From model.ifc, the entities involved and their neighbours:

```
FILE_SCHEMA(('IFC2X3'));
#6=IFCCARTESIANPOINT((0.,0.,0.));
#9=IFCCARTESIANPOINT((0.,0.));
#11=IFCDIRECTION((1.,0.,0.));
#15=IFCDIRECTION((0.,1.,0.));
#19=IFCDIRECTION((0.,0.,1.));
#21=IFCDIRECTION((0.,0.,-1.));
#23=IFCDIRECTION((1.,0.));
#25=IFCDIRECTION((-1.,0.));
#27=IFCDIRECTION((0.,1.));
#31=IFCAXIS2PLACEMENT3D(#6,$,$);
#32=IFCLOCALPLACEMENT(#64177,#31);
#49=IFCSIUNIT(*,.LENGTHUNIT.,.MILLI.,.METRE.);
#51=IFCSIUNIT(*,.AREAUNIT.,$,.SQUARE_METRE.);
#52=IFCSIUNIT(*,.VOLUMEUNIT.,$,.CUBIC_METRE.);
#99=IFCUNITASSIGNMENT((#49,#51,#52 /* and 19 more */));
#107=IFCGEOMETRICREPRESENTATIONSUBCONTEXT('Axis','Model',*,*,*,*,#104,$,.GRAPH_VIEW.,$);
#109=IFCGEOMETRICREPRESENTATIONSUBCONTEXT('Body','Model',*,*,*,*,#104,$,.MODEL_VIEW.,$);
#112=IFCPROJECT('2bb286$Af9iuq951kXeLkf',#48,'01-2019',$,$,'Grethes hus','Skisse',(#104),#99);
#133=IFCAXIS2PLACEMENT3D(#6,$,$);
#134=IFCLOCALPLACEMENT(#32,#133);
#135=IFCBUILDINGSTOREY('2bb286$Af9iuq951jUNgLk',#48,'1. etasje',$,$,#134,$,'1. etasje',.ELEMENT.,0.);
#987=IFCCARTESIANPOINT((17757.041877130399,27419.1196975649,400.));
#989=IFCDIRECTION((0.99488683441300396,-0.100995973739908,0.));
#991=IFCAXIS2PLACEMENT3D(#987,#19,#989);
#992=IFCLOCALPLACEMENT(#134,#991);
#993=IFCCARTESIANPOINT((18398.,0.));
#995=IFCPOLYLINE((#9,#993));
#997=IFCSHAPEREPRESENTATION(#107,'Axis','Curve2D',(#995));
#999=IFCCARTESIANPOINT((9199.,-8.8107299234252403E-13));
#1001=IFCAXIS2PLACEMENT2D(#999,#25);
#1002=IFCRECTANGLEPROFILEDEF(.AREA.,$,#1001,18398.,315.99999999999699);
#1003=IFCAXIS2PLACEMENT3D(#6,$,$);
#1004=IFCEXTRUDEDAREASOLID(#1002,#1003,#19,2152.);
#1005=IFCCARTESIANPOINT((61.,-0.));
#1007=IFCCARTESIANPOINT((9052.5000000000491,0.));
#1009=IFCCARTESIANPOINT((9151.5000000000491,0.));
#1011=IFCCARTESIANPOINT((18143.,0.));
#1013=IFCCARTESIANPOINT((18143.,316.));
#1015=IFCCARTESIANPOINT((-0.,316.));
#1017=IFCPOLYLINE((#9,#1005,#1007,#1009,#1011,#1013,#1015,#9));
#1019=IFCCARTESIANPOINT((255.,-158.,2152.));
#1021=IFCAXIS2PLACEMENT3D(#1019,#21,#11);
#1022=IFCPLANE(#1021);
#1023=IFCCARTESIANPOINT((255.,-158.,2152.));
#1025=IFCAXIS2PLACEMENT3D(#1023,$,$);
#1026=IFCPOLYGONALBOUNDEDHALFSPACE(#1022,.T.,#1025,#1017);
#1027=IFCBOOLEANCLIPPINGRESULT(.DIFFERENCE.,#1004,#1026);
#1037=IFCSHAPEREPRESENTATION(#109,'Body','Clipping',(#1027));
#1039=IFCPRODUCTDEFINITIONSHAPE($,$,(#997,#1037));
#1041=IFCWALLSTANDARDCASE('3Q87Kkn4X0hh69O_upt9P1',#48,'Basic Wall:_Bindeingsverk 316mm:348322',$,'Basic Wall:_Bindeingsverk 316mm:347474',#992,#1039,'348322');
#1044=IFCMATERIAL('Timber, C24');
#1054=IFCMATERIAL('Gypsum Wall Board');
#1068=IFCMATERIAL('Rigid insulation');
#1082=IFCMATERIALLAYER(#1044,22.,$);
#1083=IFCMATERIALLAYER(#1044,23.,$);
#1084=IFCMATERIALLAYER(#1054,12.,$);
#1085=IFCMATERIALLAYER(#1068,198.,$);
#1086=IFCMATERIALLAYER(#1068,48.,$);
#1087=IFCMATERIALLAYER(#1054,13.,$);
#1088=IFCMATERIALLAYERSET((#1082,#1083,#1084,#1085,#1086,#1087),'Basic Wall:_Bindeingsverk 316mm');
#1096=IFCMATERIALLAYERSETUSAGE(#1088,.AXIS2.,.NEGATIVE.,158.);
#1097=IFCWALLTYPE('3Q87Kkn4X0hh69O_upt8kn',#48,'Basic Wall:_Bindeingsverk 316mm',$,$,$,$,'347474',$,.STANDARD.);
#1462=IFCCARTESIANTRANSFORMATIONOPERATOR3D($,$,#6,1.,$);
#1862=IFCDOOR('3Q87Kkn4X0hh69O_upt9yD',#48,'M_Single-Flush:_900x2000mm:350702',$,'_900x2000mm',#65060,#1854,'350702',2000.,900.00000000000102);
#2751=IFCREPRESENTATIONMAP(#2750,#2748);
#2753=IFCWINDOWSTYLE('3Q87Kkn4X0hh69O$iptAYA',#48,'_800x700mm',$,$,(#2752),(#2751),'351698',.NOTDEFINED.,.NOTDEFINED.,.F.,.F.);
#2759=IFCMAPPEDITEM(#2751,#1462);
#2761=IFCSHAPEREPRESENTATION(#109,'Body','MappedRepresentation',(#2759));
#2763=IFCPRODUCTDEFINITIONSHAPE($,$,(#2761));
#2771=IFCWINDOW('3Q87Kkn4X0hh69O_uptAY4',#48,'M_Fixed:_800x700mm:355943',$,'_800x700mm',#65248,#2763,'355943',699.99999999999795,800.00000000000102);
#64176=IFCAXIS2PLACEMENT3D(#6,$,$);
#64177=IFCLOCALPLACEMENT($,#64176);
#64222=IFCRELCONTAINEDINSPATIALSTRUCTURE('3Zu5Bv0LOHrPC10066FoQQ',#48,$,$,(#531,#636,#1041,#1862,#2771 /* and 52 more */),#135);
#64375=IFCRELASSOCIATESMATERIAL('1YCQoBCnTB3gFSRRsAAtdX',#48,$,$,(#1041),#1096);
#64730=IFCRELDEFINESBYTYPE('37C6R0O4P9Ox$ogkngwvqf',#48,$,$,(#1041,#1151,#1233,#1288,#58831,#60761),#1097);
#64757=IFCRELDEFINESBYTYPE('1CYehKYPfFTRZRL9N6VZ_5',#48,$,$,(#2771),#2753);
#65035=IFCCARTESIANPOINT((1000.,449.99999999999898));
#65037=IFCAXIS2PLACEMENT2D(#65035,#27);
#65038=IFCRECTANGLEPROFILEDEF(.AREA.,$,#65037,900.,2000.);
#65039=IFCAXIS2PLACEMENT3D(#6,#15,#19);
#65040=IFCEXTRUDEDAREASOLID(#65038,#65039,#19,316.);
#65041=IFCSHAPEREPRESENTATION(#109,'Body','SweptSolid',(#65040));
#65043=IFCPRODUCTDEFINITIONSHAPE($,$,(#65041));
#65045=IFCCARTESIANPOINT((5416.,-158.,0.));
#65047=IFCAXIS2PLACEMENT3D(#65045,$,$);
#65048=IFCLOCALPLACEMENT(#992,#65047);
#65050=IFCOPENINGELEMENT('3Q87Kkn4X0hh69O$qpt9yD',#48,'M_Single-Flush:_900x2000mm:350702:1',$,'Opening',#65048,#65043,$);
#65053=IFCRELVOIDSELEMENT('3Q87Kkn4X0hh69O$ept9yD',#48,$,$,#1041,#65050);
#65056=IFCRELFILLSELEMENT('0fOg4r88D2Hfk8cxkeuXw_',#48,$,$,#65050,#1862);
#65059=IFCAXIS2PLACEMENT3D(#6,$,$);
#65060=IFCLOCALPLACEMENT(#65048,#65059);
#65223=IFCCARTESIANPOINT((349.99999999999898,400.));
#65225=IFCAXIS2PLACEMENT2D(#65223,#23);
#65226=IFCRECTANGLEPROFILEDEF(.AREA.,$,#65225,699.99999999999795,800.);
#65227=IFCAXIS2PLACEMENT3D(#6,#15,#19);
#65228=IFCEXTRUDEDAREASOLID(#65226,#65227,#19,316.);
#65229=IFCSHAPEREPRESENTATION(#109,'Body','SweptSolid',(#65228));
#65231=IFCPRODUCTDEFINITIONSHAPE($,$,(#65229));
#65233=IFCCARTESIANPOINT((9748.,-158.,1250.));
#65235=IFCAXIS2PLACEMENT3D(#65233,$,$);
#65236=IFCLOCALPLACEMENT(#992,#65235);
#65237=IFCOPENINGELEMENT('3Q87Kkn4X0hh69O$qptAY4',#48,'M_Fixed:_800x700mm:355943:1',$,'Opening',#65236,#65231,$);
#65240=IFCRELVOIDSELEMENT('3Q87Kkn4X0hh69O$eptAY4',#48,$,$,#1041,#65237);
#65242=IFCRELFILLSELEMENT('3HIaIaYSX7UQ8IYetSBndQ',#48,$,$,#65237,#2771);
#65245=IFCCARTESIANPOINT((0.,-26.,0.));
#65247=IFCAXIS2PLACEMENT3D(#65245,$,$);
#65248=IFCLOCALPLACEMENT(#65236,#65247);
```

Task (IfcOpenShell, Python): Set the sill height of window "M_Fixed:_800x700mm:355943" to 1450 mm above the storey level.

```python
import numpy as np
import ifcopenshell
import ifcopenshell.api.geometry
import ifcopenshell.geom
import ifcopenshell.util.element
import ifcopenshell.util.placement
import ifcopenshell.util.shape
import ifcopenshell.util.unit

model = ifcopenshell.open("model.ifc")
unit_scale = ifcopenshell.util.unit.calculate_unit_scale(model)

window = model.by_guid("3Q87Kkn4X0hh69O_uptAY4")
opening = window.FillsVoids[0].RelatingOpeningElement
storey = ifcopenshell.util.element.get_container(window, ifc_class="IfcBuildingStorey")
level = ifcopenshell.util.placement.get_local_placement(storey.ObjectPlacement)[2, 3]

# The opening's origin need not be at the sill, so measure its lowest point.
shape = ifcopenshell.geom.create_shape(ifcopenshell.geom.settings(), opening)
bottom = ifcopenshell.util.shape.get_shape_bottom_elevation(shape, shape.geometry) / unit_scale
dz = level + 1.45 / unit_scale - bottom

shift = np.array([0.0, 0.0, dz])
# The window is placed relative to its opening, so it follows when the opening moves.
matrix = ifcopenshell.util.placement.get_local_placement(opening.ObjectPlacement)
matrix[:3, 3] += shift
ifcopenshell.api.geometry.edit_object_placement(
    model, product=opening, matrix=matrix, is_si=False, should_transform_children=True
)

print(f"moved by {dz * unit_scale:+.3f} m")

model.write("model_rev.ifc")
```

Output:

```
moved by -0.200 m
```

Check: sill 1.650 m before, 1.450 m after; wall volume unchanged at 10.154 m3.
